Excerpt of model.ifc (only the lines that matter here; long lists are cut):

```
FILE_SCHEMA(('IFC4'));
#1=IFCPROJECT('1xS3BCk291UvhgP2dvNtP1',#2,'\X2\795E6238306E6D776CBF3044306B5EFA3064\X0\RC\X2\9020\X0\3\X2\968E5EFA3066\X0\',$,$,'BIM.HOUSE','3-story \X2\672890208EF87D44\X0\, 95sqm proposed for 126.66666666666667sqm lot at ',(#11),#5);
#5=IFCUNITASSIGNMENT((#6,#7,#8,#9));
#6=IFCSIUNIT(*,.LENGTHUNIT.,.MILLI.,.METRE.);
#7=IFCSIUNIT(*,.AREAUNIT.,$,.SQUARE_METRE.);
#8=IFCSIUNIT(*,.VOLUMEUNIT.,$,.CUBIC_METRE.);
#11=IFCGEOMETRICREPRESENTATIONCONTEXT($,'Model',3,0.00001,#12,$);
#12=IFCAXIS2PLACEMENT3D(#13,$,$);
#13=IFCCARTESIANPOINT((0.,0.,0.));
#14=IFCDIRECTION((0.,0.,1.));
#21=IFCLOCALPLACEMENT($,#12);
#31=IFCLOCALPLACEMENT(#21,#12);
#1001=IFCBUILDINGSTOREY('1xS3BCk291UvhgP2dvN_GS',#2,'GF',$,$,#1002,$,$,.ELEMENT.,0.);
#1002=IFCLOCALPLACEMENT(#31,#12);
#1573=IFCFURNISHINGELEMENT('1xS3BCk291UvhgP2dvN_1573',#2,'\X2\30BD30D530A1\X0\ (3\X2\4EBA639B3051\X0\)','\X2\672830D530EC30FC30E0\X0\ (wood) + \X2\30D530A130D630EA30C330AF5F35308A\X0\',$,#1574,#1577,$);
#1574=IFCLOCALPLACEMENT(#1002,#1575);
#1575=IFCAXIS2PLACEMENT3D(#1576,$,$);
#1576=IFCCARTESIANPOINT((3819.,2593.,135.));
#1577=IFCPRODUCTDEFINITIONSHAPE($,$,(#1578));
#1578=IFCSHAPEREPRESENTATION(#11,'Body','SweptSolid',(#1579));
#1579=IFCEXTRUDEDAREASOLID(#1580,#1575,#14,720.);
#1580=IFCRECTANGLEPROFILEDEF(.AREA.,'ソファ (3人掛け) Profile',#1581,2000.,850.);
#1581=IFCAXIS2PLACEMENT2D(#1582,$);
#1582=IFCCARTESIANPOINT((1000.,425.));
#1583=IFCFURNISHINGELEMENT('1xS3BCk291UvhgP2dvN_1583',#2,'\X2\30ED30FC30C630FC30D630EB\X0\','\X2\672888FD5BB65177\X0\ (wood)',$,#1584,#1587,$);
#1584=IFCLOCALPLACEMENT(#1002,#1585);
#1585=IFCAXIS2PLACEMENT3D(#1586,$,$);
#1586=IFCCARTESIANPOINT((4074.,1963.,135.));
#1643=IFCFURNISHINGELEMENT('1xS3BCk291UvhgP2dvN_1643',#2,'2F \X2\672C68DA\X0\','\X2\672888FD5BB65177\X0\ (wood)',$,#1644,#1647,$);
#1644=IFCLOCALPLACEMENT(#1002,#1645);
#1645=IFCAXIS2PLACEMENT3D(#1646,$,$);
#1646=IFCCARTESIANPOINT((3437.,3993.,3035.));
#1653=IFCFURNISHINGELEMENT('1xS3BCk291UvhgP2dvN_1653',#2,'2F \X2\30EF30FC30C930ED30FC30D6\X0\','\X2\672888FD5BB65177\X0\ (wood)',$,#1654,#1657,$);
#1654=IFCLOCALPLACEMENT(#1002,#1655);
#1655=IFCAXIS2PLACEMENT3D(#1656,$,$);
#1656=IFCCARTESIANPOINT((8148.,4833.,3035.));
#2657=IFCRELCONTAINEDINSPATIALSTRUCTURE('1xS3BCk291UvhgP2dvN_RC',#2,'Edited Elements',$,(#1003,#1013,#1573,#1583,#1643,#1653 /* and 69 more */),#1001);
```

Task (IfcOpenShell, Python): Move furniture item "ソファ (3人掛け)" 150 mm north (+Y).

```python
import ifcopenshell
import ifcopenshell.api.geometry
import ifcopenshell.util.placement

model = ifcopenshell.open("model.ifc")

item = model.by_guid("1xS3BCk291UvhgP2dvN_1573")
matrix = ifcopenshell.util.placement.get_local_placement(item.ObjectPlacement)
matrix[1, 3] += 150.0
ifcopenshell.api.geometry.edit_object_placement(model, product=item, matrix=matrix, is_si=False)

print(ifcopenshell.util.placement.get_local_placement(item.ObjectPlacement).round(3) + 0.0)

model.write("model-out.ifc")
```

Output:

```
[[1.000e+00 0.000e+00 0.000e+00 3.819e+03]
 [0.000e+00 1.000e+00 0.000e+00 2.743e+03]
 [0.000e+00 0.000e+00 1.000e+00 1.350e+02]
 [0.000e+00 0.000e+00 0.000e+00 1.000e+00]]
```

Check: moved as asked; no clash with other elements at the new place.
